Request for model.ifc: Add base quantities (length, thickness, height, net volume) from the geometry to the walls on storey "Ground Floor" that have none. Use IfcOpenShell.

First a look at what the model holds.

```python
import ifcopenshell
import ifcopenshell.util.element
import ifcopenshell.util.unit

model = ifcopenshell.open("model.ifc")
print(model.schema)
for unit_type in ("LENGTHUNIT", "AREAUNIT", "VOLUMEUNIT"):
    print(unit_type, ifcopenshell.util.unit.calculate_unit_scale(model, unit_type))
storey = next(s for s in model.by_type("IfcBuildingStorey") if s.Name == "Ground Floor")
walls = [e for e in ifcopenshell.util.element.get_decomposition(storey) if e.is_a("IfcWall")]
for e in sorted(walls, key=lambda e: e.id()):
    print(e.id(), e.is_a(), e.Name, list(ifcopenshell.util.element.get_psets(e, qtos_only=True)), sep=" | ")
```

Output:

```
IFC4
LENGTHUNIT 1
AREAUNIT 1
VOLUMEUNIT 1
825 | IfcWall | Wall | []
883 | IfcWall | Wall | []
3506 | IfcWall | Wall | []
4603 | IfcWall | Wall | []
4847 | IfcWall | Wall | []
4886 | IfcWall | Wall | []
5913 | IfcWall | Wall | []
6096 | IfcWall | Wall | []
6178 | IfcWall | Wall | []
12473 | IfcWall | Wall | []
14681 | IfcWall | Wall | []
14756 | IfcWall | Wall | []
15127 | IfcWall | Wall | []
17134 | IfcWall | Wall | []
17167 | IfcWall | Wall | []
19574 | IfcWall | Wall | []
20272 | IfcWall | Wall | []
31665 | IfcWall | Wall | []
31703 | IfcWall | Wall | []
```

```python
import ifcopenshell
import ifcopenshell.api.pset
import ifcopenshell.geom
import ifcopenshell.util.element
import ifcopenshell.util.shape
import ifcopenshell.util.unit

model = ifcopenshell.open("model.ifc")
unit_scale = ifcopenshell.util.unit.calculate_unit_scale(model)
volume_scale = ifcopenshell.util.unit.calculate_unit_scale(model, "VOLUMEUNIT")
settings = ifcopenshell.geom.settings()

storey = next(s for s in model.by_type("IfcBuildingStorey") if s.Name == "Ground Floor")
walls = [e for e in ifcopenshell.util.element.get_decomposition(storey) if e.is_a("IfcWall")]

for e in sorted(walls, key=lambda e: e.id()):
    if ifcopenshell.util.element.get_psets(e, qtos_only=True, should_inherit=False):
        continue
    # Geometry comes back in metres, in the element's own axes.
    shape = ifcopenshell.geom.create_shape(settings, e)
    values = {
        "Length": ifcopenshell.util.shape.get_x(shape.geometry) / unit_scale,
        "Width": ifcopenshell.util.shape.get_y(shape.geometry) / unit_scale,
        "Height": ifcopenshell.util.shape.get_z(shape.geometry) / unit_scale,
        "NetVolume": ifcopenshell.util.shape.get_volume(shape.geometry) / volume_scale,
    }
    qto = ifcopenshell.api.pset.add_qto(model, product=e, name="Qto_WallBaseQuantities")
    ifcopenshell.api.pset.edit_qto(model, qto=qto, properties=values)
    print(e.id(), {k: round(v, 3) for k, v in values.items()})

model.write("model_rev.ifc")
```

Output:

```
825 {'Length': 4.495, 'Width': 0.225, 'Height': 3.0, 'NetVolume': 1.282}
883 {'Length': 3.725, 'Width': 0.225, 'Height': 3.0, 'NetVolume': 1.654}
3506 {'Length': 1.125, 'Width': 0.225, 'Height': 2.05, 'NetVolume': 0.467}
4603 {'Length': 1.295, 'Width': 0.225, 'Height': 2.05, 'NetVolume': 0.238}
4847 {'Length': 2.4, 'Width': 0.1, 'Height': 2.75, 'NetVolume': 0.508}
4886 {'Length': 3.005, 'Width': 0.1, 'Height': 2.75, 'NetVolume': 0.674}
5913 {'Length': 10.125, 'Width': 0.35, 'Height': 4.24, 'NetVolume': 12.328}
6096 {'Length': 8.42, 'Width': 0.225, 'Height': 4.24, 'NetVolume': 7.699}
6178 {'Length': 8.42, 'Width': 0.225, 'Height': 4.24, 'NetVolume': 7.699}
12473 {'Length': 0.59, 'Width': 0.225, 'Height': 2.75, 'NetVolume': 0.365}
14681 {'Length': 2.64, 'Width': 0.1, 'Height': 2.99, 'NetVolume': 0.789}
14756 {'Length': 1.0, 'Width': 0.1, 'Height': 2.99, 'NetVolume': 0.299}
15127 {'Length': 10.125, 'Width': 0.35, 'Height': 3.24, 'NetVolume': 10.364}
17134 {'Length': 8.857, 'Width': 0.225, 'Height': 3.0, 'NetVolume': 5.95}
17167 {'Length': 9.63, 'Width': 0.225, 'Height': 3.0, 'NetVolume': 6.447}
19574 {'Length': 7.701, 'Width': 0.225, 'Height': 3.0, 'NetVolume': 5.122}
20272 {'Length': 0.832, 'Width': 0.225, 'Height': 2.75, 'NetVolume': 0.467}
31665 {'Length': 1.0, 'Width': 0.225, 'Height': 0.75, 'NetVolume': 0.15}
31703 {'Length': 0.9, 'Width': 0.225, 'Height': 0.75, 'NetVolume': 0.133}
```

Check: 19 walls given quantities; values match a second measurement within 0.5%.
